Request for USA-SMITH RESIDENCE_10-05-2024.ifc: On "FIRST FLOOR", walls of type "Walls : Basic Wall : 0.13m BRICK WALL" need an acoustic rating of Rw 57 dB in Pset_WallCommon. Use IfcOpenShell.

First a look at what the model holds.

```python
import ifcopenshell
import ifcopenshell.util.element

model = ifcopenshell.open("USA-SMITH RESIDENCE_10-05-2024.ifc")
print(model.schema)
storey = next(s for s in model.by_type("IfcBuildingStorey") if s.Name == "FIRST FLOOR")
walls = [e for e in ifcopenshell.util.element.get_decomposition(storey) if e.is_a("IfcWall")]
seen = {}
for e in walls:
    element_type = ifcopenshell.util.element.get_type(e)
    key = (element_type.Name if element_type != e and element_type else None, ifcopenshell.util.element.get_pset(e, "Pset_WallCommon", "AcousticRating"))
    seen[key] = seen.get(key, 0) + 1
for (name, value), count in sorted(seen.items(), key=str):
    print(count, "x", name, "|", value)
```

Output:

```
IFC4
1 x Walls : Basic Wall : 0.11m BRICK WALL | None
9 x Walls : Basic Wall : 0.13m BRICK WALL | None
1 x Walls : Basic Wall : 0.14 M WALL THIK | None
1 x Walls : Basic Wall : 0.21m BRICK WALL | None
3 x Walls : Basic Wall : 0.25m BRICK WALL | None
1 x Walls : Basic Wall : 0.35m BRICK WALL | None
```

```python
import ifcopenshell
import ifcopenshell.api.pset
import ifcopenshell.util.element

model = ifcopenshell.open("USA-SMITH RESIDENCE_10-05-2024.ifc")

storey = next(s for s in model.by_type("IfcBuildingStorey") if s.Name == "FIRST FLOOR")
walls = [e for e in ifcopenshell.util.element.get_decomposition(storey) if e.is_a("IfcWall")]

count = 0
for e in walls:
    element_type = ifcopenshell.util.element.get_type(e)
    if element_type in (None, e) or element_type.Name != "Walls : Basic Wall : 0.13m BRICK WALL":
        continue
    # add_pset returns the element's existing set when there is one.
    pset = ifcopenshell.api.pset.add_pset(model, product=e, name="Pset_WallCommon")
    ifcopenshell.api.pset.edit_pset(model, pset=pset, properties={"AcousticRating": "Rw 57 dB"})
    count += 1

print(count, "walls updated")

model.write("USA-SMITH RESIDENCE_10-05-2024_v2.ifc")
```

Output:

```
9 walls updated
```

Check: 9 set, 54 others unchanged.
